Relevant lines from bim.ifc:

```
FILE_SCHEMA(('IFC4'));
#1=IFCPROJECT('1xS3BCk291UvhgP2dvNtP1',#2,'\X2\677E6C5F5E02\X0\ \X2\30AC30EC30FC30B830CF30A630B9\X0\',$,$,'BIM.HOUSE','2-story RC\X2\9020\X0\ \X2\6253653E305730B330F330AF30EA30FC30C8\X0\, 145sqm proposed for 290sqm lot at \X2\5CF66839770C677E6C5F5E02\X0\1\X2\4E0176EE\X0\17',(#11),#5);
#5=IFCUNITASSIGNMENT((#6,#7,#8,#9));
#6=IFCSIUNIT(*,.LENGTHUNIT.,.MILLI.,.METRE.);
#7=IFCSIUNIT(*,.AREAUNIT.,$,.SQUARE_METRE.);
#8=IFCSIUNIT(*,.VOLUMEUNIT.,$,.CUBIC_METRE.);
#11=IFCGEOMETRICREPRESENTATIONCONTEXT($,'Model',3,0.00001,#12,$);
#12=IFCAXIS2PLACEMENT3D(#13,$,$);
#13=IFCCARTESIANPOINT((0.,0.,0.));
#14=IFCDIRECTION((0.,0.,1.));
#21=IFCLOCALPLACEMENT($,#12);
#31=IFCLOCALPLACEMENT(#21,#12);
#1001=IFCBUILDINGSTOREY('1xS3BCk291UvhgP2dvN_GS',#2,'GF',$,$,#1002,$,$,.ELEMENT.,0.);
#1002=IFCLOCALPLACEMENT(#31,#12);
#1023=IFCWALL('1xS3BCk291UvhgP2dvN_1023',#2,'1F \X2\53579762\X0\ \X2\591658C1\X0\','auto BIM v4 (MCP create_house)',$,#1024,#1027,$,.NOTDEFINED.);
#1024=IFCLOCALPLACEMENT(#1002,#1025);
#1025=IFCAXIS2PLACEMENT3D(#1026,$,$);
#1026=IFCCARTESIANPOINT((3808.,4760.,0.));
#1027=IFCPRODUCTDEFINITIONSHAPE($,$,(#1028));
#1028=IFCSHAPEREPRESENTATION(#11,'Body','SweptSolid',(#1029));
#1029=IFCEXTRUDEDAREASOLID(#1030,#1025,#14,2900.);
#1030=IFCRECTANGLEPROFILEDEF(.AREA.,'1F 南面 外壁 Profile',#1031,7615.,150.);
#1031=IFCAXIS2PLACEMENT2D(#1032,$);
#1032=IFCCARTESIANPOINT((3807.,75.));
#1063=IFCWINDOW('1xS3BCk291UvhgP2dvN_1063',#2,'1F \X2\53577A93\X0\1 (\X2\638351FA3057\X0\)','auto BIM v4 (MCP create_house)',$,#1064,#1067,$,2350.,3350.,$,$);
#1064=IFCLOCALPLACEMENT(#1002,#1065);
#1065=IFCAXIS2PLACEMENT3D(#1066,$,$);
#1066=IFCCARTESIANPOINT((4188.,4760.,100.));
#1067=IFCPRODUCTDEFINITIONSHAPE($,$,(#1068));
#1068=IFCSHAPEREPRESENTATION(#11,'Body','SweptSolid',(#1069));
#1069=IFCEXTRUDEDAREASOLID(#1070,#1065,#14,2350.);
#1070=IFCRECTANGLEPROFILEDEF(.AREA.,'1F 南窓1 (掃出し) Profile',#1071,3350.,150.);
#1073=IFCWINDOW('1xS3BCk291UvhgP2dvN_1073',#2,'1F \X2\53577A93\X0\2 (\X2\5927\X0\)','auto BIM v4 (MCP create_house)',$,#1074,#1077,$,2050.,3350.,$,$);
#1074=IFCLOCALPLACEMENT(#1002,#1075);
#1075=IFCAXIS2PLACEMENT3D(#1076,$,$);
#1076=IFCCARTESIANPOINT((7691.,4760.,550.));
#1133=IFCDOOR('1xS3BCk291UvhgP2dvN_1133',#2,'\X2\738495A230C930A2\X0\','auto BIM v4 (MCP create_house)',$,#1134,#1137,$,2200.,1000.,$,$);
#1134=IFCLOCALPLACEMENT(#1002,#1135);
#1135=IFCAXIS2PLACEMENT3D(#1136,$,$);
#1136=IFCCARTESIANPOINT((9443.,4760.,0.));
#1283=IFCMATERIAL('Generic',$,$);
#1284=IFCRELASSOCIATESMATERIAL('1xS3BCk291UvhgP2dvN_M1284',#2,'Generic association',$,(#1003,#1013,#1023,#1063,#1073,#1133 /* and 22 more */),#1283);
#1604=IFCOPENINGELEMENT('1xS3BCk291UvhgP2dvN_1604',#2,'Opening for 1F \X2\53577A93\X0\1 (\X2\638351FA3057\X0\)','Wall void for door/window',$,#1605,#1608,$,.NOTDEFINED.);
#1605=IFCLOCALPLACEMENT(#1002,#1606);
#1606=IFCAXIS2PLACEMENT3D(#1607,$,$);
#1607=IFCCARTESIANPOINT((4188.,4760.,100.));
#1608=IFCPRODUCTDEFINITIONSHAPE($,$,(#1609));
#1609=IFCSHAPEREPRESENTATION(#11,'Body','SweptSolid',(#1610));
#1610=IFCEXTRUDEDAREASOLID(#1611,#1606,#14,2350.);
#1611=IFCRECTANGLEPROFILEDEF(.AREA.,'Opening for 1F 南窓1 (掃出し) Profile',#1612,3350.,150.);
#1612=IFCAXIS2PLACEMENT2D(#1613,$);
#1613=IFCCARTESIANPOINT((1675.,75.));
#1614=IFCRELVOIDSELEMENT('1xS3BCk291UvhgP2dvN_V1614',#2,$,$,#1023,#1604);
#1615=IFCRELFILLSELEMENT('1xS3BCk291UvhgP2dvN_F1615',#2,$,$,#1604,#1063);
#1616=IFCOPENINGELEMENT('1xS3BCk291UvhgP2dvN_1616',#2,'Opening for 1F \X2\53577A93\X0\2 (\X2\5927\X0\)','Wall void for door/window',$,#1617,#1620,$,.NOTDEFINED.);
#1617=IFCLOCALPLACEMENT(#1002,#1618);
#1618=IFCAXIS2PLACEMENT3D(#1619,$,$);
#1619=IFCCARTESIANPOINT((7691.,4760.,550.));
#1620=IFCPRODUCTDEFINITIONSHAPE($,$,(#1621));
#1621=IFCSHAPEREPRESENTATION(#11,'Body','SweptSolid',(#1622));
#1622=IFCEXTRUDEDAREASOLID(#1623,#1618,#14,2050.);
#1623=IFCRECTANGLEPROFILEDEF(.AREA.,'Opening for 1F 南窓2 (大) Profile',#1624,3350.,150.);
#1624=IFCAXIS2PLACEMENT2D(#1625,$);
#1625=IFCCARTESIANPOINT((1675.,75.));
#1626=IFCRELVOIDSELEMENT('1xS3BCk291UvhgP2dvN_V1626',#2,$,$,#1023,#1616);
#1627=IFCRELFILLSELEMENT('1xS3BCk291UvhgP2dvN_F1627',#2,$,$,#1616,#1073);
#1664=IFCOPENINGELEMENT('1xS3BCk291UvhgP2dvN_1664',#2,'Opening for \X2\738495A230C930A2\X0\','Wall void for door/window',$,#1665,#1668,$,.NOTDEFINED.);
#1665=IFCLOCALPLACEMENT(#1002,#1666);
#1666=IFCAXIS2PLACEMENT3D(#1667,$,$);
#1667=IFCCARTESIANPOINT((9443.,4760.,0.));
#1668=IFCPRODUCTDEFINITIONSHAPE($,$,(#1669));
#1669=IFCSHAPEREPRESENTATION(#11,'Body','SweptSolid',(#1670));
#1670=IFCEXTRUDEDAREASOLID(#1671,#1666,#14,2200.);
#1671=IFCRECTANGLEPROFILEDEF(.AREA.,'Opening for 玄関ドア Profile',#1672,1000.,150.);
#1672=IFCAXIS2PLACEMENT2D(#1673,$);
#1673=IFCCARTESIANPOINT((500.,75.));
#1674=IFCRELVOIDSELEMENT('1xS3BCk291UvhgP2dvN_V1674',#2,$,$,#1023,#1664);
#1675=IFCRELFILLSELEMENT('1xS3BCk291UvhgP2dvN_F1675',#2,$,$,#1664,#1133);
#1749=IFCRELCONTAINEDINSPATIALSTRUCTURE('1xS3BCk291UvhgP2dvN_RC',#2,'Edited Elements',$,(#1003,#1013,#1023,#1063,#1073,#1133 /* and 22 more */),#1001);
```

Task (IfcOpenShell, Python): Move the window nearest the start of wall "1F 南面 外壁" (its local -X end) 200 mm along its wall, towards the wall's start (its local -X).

```python
import ifcopenshell
import ifcopenshell.api.geometry
import ifcopenshell.util.placement
import ifcopenshell.util.unit

model = ifcopenshell.open("bim.ifc")
unit_scale = ifcopenshell.util.unit.calculate_unit_scale(model)

window = model.by_guid("1xS3BCk291UvhgP2dvN_1063")
opening = window.FillsVoids[0].RelatingOpeningElement
wall = opening.VoidsElements[0].RelatingBuildingElement

wall_matrix = ifcopenshell.util.placement.get_local_placement(wall.ObjectPlacement)
shift = wall_matrix[:3, 0] * -0.2 / unit_scale
before = ifcopenshell.util.placement.get_local_placement(window.ObjectPlacement)[:3, 3].copy()

# The window is not placed relative to its opening, so move both.
for product in (opening, window):
    matrix = ifcopenshell.util.placement.get_local_placement(product.ObjectPlacement)
    matrix[:3, 3] += shift
    ifcopenshell.api.geometry.edit_object_placement(model, product=product, matrix=matrix, is_si=False)

after = ifcopenshell.util.placement.get_local_placement(window.ObjectPlacement)[:3, 3]
print("window moved by", (after - before).round(3) + 0.0)

model.write("bim_v2.ifc")
```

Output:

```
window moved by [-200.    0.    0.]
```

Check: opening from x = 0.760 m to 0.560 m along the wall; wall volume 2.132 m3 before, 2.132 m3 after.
